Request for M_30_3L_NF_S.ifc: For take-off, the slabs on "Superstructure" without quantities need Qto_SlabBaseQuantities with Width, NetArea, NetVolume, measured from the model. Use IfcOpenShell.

First a look at what the model holds.

```python
import ifcopenshell
import ifcopenshell.util.element
import ifcopenshell.util.unit

model = ifcopenshell.open("M_30_3L_NF_S.ifc")
print(model.schema)
for unit_type in ("LENGTHUNIT", "AREAUNIT", "VOLUMEUNIT"):
    print(unit_type, ifcopenshell.util.unit.calculate_unit_scale(model, unit_type))
storey = next(s for s in model.by_type("IfcBuildingStorey") if s.Name == "Superstructure")
slabs = [e for e in ifcopenshell.util.element.get_decomposition(storey) if e.is_a("IfcSlab")]
for e in sorted(slabs, key=lambda e: e.id()):
    print(e.id(), e.is_a(), e.Name, list(ifcopenshell.util.element.get_psets(e, qtos_only=True)), sep=" | ")
```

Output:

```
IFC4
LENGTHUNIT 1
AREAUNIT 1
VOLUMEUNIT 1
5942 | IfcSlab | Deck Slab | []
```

```python
import ifcopenshell
import ifcopenshell.api.pset
import ifcopenshell.geom
import ifcopenshell.util.element
import ifcopenshell.util.shape
import ifcopenshell.util.unit

model = ifcopenshell.open("M_30_3L_NF_S.ifc")
unit_scale = ifcopenshell.util.unit.calculate_unit_scale(model)
area_scale = ifcopenshell.util.unit.calculate_unit_scale(model, "AREAUNIT")
volume_scale = ifcopenshell.util.unit.calculate_unit_scale(model, "VOLUMEUNIT")
settings = ifcopenshell.geom.settings()

storey = next(s for s in model.by_type("IfcBuildingStorey") if s.Name == "Superstructure")
slabs = [e for e in ifcopenshell.util.element.get_decomposition(storey) if e.is_a("IfcSlab")]

for e in sorted(slabs, key=lambda e: e.id()):
    if ifcopenshell.util.element.get_psets(e, qtos_only=True, should_inherit=False):
        continue
    # Geometry comes back in metres, in the element's own axes.
    shape = ifcopenshell.geom.create_shape(settings, e)
    values = {
        "Width": ifcopenshell.util.shape.get_z(shape.geometry) / unit_scale,
        "NetArea": ifcopenshell.util.shape.get_footprint_area(shape.geometry) / area_scale,
        "NetVolume": ifcopenshell.util.shape.get_volume(shape.geometry) / volume_scale,
    }
    qto = ifcopenshell.api.pset.add_qto(model, product=e, name="Qto_SlabBaseQuantities")
    ifcopenshell.api.pset.edit_qto(model, qto=qto, properties=values)
    print(e.id(), {k: round(v, 3) for k, v in values.items()})

model.write("M_30_3L_NF_S-out.ifc")
```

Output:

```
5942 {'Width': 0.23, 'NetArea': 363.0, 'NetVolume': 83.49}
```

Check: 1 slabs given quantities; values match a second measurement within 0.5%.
